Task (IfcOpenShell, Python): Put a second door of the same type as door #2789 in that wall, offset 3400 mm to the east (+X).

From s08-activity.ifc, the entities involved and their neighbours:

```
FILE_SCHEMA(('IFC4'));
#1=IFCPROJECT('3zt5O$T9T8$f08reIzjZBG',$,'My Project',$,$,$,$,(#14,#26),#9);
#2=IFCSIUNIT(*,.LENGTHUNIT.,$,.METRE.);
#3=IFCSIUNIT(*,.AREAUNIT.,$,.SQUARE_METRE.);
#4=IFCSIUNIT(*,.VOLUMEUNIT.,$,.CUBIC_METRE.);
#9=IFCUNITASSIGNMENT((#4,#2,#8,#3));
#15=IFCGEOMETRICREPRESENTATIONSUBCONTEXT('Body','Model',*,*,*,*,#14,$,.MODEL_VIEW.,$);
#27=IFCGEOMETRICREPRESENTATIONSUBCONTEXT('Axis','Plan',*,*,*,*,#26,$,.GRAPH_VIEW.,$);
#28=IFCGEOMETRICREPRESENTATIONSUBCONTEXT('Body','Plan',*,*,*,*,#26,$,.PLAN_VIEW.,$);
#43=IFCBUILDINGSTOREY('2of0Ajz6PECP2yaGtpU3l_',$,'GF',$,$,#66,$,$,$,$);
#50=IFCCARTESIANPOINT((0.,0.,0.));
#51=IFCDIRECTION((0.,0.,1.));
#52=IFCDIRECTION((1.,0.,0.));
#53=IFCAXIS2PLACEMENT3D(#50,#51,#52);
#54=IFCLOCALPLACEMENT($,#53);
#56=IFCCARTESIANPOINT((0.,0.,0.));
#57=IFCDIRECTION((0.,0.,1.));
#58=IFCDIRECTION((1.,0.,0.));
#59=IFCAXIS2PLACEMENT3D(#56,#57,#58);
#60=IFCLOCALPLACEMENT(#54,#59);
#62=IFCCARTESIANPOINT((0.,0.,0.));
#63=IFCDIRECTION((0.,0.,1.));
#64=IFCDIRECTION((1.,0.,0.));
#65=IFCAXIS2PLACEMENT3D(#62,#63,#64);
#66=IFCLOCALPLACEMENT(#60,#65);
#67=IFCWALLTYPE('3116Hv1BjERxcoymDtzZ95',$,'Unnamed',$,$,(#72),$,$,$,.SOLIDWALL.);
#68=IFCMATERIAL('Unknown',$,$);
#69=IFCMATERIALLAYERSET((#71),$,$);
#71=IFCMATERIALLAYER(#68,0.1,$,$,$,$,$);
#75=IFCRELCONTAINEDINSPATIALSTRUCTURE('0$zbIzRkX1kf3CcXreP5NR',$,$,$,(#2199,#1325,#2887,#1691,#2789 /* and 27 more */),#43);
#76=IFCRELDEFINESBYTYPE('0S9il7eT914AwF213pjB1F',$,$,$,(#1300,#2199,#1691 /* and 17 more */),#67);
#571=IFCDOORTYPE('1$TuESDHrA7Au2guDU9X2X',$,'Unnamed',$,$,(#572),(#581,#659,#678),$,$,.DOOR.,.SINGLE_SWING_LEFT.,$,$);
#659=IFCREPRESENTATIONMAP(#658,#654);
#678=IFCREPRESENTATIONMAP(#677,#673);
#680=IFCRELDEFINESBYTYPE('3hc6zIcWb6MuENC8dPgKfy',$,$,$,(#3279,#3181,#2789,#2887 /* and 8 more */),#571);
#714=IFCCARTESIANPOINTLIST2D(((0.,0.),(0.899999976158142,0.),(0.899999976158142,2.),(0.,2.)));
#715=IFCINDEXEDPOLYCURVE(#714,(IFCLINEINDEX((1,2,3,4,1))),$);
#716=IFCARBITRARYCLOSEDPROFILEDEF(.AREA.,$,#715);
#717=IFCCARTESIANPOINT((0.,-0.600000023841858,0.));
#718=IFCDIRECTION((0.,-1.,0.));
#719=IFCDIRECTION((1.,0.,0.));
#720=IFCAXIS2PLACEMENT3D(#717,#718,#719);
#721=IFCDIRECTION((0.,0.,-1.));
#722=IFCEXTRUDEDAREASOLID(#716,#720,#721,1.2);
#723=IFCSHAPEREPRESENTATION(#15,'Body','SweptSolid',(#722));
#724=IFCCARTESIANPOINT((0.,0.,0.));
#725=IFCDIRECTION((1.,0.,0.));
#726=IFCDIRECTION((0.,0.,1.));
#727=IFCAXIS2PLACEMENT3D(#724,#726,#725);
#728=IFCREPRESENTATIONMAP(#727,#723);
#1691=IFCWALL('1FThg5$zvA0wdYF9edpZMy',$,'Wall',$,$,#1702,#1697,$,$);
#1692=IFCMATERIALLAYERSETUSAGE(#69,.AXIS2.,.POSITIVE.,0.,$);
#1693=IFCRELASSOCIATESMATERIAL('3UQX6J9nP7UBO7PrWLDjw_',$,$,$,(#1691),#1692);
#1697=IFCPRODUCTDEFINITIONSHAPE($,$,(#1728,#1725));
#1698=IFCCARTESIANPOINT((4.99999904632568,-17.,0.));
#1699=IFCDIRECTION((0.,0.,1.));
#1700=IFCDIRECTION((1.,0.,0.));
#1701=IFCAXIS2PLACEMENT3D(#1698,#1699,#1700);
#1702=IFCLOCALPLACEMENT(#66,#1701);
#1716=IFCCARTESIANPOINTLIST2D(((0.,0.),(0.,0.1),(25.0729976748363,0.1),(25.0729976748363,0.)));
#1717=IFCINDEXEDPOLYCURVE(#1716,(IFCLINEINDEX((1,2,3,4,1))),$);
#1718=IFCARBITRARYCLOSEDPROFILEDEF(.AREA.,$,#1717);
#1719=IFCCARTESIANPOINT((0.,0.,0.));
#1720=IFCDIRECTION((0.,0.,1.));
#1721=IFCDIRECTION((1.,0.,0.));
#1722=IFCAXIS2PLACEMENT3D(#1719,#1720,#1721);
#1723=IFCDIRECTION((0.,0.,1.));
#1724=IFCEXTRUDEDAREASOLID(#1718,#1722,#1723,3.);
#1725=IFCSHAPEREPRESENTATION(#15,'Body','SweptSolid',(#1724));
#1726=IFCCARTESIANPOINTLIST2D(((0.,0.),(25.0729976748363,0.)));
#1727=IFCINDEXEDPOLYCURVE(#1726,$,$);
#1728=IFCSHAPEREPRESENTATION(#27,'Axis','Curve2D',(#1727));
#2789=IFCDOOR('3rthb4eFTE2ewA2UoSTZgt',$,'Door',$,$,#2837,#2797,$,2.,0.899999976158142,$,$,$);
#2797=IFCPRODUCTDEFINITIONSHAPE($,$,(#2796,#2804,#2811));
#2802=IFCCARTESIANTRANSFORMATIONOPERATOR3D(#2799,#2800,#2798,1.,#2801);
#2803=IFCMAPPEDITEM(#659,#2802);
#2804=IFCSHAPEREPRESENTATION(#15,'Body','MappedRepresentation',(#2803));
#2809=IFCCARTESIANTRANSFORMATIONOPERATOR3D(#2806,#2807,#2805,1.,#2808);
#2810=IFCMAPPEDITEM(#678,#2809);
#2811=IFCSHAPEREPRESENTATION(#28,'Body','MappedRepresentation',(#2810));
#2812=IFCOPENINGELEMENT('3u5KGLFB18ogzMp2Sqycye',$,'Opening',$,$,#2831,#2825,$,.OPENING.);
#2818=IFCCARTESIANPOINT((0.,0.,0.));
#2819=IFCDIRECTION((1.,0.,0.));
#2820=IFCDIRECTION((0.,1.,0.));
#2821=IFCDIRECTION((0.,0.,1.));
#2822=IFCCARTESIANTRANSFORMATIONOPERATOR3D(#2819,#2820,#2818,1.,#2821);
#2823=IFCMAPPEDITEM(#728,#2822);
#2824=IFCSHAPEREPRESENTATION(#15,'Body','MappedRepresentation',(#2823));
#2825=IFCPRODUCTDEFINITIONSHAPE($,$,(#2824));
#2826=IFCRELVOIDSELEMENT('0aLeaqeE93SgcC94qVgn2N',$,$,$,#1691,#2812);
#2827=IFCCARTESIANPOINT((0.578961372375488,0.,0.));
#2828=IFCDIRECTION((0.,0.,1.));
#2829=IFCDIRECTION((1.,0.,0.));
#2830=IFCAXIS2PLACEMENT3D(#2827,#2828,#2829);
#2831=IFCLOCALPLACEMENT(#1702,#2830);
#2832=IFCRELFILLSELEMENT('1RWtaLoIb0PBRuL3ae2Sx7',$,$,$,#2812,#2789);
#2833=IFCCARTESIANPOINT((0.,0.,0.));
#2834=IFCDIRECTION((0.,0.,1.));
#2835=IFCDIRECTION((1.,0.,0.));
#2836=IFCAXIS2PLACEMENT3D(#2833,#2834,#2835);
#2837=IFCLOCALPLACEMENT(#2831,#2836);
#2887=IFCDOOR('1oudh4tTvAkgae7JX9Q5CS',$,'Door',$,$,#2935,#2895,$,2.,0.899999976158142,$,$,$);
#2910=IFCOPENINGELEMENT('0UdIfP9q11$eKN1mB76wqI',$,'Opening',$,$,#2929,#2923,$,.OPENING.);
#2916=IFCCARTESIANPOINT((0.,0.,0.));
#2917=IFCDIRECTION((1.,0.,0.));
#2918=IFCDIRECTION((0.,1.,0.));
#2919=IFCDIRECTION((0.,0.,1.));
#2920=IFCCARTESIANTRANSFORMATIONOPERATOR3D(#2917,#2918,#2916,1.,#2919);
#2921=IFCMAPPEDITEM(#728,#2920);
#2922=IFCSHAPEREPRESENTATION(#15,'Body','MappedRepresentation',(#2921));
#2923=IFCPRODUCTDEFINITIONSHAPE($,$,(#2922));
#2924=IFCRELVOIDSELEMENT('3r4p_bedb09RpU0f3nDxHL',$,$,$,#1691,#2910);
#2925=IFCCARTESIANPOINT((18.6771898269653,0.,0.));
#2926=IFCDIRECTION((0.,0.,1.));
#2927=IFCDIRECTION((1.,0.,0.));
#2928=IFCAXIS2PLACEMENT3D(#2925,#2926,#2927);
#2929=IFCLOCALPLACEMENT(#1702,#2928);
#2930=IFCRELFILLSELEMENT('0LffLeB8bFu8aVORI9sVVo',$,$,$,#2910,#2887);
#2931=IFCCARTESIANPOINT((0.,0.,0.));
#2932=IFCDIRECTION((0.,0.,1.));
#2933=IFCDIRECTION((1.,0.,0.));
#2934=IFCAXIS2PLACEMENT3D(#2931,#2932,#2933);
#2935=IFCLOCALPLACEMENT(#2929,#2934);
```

```python
import ifcopenshell
import ifcopenshell.api.feature
import ifcopenshell.api.geometry
import ifcopenshell.api.root
import ifcopenshell.geom
import ifcopenshell.util.element
import ifcopenshell.util.placement
import ifcopenshell.util.shape
import ifcopenshell.util.unit

model = ifcopenshell.open("s08-activity.ifc")
unit_scale = ifcopenshell.util.unit.calculate_unit_scale(model)
settings = ifcopenshell.geom.settings()


def volume(element):
    """Net volume in cubic metres, openings subtracted."""
    shape = ifcopenshell.geom.create_shape(settings, element)
    return ifcopenshell.util.shape.get_volume(shape.geometry)


door = model.by_guid("3rthb4eFTE2ewA2UoSTZgt")
opening = door.FillsVoids[0].RelatingOpeningElement
wall = opening.VoidsElements[0].RelatingBuildingElement
before = volume(wall)
shift = ifcopenshell.util.placement.get_local_placement(wall.ObjectPlacement)[:3, 0] * 3.4 / unit_scale

# copy_class copies the void relationship, type, container and properties, but no geometry.
new_opening = ifcopenshell.api.root.copy_class(model, product=opening)
new_opening.Representation = ifcopenshell.util.element.copy_deep(
    model, opening.Representation, exclude=["IfcGeometricRepresentationContext", "IfcRepresentationMap"]
)
new_door = ifcopenshell.api.root.copy_class(model, product=door)
new_door.Representation = ifcopenshell.util.element.copy_deep(
    model, door.Representation, exclude=["IfcGeometricRepresentationContext", "IfcRepresentationMap"]
)
ifcopenshell.api.feature.add_filling(model, opening=new_opening, element=new_door)

for old, new in ((opening, new_opening), (door, new_door)):
    matrix = ifcopenshell.util.placement.get_local_placement(old.ObjectPlacement)
    matrix[:3, 3] += shift
    ifcopenshell.api.geometry.edit_object_placement(model, product=new, matrix=matrix, is_si=False)

after = volume(wall)

print(f"wall volume {before:.3f} -> {after:.3f} m3")

model.write("s08-activity_v2.ifc")
```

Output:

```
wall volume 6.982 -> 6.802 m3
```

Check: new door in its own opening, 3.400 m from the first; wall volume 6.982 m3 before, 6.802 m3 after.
